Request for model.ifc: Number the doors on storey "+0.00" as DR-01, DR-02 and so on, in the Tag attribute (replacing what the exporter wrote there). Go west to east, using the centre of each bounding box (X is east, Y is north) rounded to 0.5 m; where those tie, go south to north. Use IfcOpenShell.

First a look at what the model holds.

```python
import ifcopenshell
import ifcopenshell.util.element
import ifcopenshell.util.placement

model = ifcopenshell.open("model.ifc")
print(model.schema)
storey = next(s for s in model.by_type("IfcBuildingStorey") if s.Name == "+0.00")
doors = [e for e in ifcopenshell.util.element.get_decomposition(storey) if e.is_a("IfcDoor")]
for e in sorted(doors, key=lambda e: e.id()):
    origin = ifcopenshell.util.placement.get_local_placement(e.ObjectPlacement)[:3, 3]
    print(e.id(), e.Tag, e.Name, origin.round(2) + 0.0, sep=" | ")
```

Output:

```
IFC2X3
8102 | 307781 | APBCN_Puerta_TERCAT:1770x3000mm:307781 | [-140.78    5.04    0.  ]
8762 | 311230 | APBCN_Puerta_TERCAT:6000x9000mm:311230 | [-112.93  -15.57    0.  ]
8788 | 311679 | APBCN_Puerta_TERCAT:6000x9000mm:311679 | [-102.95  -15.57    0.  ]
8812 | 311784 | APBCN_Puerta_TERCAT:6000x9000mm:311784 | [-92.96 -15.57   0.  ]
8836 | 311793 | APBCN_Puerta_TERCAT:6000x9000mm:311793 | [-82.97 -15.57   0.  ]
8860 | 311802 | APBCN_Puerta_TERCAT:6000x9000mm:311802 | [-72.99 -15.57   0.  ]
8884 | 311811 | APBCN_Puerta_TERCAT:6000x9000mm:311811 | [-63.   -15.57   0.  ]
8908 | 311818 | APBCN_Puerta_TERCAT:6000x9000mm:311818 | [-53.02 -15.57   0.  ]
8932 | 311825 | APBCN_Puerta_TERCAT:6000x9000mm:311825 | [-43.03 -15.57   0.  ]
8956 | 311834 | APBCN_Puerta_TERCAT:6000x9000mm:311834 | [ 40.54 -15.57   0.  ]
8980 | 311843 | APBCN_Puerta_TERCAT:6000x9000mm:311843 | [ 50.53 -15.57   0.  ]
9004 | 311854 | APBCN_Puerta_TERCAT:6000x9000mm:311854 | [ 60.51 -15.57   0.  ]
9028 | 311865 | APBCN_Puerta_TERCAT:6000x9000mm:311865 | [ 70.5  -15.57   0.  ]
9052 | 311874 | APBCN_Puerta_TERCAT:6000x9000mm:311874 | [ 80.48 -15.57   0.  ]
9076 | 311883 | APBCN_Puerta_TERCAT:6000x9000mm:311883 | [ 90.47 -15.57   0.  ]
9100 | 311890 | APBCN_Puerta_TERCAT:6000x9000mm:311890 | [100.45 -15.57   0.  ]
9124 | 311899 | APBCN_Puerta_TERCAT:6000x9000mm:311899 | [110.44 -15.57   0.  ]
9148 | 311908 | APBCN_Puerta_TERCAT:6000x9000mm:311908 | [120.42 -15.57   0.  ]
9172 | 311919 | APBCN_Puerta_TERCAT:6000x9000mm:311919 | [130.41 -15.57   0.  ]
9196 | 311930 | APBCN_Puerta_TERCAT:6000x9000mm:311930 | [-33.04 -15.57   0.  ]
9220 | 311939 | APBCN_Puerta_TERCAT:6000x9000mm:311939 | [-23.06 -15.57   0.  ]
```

```python
import ifcopenshell
import ifcopenshell.geom
import ifcopenshell.util.element
import ifcopenshell.util.shape

model = ifcopenshell.open("model.ifc")
settings = ifcopenshell.geom.settings()
settings.set("use-world-coords", True)


def centre(element):
    shape = ifcopenshell.geom.create_shape(settings, element)
    return ifcopenshell.util.shape.get_bbox_centroid(shape.geometry)


storey = next(s for s in model.by_type("IfcBuildingStorey") if s.Name == "+0.00")
doors = [e for e in ifcopenshell.util.element.get_decomposition(storey) if e.is_a("IfcDoor")]

# Insertion points can sit at a corner or the storey origin, so sort by the geometry (in metres).
centres = {e: centre(e) for e in doors}
doors.sort(key=lambda e: (round(centres[e][0] / 0.5), centres[e][1]))

for i, e in enumerate(doors, start=1):
    number = f"DR-{i:02d}"
    e.Tag = number
    print(e.id(), number)

model.write("model_edited.ifc")
```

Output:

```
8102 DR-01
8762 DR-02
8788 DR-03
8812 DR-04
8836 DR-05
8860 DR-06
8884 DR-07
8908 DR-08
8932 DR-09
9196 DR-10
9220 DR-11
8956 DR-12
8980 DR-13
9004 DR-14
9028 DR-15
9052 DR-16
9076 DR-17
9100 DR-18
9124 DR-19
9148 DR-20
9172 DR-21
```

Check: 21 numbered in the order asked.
